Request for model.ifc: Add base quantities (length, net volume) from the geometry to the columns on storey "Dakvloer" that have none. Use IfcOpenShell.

First a look at what the model holds.

```python
import ifcopenshell
import ifcopenshell.util.element
import ifcopenshell.util.unit

model = ifcopenshell.open("model.ifc")
print(model.schema)
for unit_type in ("LENGTHUNIT", "AREAUNIT", "VOLUMEUNIT"):
    print(unit_type, ifcopenshell.util.unit.calculate_unit_scale(model, unit_type))
storey = next(s for s in model.by_type("IfcBuildingStorey") if s.Name == "Dakvloer")
columns = [e for e in ifcopenshell.util.element.get_decomposition(storey) if e.is_a("IfcColumn")]
for e in sorted(columns, key=lambda e: e.id()):
    print(e.id(), e.is_a(), e.Name, list(ifcopenshell.util.element.get_psets(e, qtos_only=True)), sep=" | ")
```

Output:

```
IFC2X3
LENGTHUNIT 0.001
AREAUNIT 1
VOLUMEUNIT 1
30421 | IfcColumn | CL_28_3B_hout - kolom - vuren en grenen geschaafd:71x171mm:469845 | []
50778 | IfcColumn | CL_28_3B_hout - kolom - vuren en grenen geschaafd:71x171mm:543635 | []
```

```python
import ifcopenshell
import ifcopenshell.api.pset
import ifcopenshell.geom
import ifcopenshell.util.element
import ifcopenshell.util.shape
import ifcopenshell.util.unit

model = ifcopenshell.open("model.ifc")
unit_scale = ifcopenshell.util.unit.calculate_unit_scale(model)
volume_scale = ifcopenshell.util.unit.calculate_unit_scale(model, "VOLUMEUNIT")
settings = ifcopenshell.geom.settings()

storey = next(s for s in model.by_type("IfcBuildingStorey") if s.Name == "Dakvloer")
columns = [e for e in ifcopenshell.util.element.get_decomposition(storey) if e.is_a("IfcColumn")]

for e in sorted(columns, key=lambda e: e.id()):
    if ifcopenshell.util.element.get_psets(e, qtos_only=True, should_inherit=False):
        continue
    # Geometry comes back in metres, in the element's own axes.
    shape = ifcopenshell.geom.create_shape(settings, e)
    values = {
        "Length": ifcopenshell.util.shape.get_z(shape.geometry) / unit_scale,
        "NetVolume": ifcopenshell.util.shape.get_volume(shape.geometry) / volume_scale,
    }
    qto = ifcopenshell.api.pset.add_qto(model, product=e, name="BaseQuantities")
    ifcopenshell.api.pset.edit_qto(model, qto=qto, properties=values)
    print(e.id(), {k: round(v, 3) for k, v in values.items()})

model.write("model_edited.ifc")
```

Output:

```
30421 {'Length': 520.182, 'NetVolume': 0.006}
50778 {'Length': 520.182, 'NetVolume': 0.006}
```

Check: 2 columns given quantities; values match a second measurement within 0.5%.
